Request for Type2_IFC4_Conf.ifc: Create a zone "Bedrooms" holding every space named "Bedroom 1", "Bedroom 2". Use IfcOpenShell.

First a look at what the model holds.

```python
import ifcopenshell

model = ifcopenshell.open("Type2_IFC4_Conf.ifc")
print(model.schema)
seen = {}
for space in model.by_type("IfcSpace"):
    seen[space.LongName] = seen.get(space.LongName, 0) + 1
for name, count in sorted(seen.items(), key=str):
    print(count, "x", name)
print("zones:", [z.Name for z in model.by_type("IfcZone")][:20])
```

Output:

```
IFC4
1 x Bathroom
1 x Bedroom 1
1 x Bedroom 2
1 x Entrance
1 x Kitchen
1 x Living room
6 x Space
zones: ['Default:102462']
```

```python
import ifcopenshell
import ifcopenshell.api.group
import ifcopenshell.api.root

model = ifcopenshell.open("Type2_IFC4_Conf.ifc")

names = {"Bedroom 1", "Bedroom 2"}
spaces = [s for s in model.by_type("IfcSpace") if s.LongName in names]

zone = ifcopenshell.api.root.create_entity(model, ifc_class="IfcZone", name="Bedrooms")
ifcopenshell.api.group.assign_group(model, products=spaces, group=zone)
print(len(spaces), "spaces in", zone.Name)

model.write("Type2_IFC4_Conf_rev.ifc")
```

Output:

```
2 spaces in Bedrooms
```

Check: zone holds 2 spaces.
